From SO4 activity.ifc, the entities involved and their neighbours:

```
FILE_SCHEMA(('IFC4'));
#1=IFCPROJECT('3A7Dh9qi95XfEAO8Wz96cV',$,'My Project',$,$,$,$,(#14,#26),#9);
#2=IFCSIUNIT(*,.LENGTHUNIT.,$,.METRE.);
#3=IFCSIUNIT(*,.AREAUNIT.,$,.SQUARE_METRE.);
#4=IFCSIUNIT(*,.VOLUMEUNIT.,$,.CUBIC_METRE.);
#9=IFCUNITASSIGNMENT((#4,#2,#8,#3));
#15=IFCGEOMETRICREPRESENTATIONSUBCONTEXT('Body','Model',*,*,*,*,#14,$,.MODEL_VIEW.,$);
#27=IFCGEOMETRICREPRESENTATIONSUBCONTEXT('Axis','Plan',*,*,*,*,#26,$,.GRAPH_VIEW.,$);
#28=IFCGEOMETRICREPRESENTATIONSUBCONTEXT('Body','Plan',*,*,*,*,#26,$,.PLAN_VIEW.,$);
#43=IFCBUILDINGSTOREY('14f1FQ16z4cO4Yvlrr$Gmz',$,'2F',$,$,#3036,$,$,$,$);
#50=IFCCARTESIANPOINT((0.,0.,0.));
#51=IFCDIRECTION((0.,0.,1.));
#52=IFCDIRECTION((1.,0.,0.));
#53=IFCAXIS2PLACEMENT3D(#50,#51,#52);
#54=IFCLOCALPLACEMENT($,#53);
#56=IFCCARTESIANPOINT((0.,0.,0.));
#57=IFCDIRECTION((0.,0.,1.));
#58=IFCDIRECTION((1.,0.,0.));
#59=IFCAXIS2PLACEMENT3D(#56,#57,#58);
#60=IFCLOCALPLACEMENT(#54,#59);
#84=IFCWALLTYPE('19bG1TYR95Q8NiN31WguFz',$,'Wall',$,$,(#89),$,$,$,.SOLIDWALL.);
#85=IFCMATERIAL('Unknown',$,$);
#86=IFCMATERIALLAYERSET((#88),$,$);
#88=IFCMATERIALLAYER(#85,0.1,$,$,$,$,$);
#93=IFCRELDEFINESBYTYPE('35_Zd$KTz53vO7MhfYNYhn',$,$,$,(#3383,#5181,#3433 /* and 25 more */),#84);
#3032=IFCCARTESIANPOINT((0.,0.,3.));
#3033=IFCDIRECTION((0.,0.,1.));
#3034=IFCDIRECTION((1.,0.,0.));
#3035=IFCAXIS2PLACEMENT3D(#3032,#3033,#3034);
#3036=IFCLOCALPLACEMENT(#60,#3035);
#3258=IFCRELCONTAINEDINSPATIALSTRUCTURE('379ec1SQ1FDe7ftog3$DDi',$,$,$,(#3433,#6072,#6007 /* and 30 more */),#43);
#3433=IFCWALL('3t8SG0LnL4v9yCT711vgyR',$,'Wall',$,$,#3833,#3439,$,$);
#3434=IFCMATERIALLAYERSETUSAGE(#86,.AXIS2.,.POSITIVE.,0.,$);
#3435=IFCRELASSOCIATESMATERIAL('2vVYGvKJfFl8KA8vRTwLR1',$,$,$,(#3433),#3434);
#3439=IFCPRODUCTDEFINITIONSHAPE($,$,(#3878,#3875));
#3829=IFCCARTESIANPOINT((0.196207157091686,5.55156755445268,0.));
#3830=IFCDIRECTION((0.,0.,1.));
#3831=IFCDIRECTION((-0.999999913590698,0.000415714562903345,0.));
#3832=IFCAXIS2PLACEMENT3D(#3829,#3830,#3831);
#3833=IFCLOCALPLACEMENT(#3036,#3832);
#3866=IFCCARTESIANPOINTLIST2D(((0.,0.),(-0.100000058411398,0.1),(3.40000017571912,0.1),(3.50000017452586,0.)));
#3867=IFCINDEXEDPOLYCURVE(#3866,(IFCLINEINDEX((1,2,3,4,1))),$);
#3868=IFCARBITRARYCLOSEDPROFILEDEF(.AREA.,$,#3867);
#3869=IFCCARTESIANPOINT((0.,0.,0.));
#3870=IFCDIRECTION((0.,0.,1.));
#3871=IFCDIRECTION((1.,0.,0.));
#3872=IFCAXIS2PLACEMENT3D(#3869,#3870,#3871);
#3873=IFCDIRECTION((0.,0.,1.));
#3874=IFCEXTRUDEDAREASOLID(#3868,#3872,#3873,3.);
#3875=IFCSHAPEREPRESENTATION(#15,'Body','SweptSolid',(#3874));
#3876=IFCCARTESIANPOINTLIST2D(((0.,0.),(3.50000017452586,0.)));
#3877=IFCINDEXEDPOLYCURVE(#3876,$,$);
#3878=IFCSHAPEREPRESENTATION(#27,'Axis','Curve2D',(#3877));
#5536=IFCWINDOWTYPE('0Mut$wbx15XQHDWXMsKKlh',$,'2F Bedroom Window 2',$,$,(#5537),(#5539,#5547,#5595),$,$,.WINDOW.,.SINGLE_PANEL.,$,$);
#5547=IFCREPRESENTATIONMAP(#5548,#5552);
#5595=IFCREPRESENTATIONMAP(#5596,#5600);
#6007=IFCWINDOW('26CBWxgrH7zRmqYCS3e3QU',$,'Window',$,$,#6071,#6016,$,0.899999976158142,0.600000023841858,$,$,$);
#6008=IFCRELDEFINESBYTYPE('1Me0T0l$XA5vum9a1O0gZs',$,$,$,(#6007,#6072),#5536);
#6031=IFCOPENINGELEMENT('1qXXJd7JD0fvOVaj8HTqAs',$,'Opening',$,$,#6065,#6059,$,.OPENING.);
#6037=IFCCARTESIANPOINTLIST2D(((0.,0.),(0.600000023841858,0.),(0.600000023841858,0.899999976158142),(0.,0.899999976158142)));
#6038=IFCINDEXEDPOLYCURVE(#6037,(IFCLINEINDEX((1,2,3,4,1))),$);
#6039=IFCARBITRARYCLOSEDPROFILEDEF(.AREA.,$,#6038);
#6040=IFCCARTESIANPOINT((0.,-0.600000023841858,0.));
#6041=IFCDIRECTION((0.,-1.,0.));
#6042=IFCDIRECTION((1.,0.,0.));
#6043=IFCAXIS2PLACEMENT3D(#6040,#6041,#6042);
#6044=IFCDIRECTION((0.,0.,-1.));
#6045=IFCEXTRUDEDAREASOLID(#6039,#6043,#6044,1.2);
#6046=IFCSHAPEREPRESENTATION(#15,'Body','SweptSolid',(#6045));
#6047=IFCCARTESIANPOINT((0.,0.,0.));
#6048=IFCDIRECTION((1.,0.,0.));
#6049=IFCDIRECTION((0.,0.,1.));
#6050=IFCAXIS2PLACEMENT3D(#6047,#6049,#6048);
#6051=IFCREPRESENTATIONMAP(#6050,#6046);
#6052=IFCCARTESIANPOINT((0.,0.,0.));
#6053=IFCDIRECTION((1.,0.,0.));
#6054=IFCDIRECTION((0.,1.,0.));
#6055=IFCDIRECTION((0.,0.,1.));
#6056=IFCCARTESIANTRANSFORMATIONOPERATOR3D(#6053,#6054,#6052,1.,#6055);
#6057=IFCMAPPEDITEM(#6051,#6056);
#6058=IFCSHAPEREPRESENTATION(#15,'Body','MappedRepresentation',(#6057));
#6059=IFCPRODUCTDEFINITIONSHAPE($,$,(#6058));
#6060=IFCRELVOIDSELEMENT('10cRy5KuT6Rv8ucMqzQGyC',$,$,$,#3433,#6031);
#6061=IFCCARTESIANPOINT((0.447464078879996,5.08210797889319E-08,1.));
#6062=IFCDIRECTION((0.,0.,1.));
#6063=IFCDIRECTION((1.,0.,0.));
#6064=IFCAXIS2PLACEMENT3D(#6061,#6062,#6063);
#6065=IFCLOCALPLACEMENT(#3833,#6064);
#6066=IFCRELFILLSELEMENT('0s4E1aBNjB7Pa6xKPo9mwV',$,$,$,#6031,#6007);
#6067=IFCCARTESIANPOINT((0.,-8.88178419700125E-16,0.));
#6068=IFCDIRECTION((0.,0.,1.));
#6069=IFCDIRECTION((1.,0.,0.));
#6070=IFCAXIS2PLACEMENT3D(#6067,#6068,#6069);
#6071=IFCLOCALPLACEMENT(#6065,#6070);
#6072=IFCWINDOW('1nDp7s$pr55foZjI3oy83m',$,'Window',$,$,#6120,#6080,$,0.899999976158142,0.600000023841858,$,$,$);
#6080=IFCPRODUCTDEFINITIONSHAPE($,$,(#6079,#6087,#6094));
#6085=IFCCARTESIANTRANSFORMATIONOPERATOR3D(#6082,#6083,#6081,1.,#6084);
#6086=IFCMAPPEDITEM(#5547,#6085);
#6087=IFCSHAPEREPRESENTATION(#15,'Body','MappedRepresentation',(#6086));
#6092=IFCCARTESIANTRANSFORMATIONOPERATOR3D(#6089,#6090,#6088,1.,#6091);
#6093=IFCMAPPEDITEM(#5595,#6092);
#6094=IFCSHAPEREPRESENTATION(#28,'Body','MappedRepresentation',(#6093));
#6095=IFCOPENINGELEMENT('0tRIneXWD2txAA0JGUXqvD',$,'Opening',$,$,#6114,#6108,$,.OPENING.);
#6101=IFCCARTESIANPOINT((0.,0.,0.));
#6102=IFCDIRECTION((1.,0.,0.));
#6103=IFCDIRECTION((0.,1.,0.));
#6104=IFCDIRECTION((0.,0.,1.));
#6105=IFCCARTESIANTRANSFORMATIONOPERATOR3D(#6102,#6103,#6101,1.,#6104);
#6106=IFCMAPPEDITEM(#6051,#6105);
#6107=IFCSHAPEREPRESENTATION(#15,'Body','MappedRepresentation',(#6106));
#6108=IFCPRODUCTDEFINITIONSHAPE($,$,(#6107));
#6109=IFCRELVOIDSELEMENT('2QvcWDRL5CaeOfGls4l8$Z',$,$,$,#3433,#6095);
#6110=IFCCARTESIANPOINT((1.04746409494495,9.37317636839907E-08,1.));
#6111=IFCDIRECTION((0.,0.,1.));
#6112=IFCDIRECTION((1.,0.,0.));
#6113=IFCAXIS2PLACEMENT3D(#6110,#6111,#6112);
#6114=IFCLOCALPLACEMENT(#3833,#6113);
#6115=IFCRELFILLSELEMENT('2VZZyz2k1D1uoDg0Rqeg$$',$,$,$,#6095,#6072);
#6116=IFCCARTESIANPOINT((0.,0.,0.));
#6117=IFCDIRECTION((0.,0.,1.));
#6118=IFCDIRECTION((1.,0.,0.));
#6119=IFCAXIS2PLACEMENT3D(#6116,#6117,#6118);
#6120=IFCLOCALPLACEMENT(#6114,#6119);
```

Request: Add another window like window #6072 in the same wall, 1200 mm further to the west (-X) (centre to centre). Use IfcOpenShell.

```python
import ifcopenshell
import ifcopenshell.api.feature
import ifcopenshell.api.geometry
import ifcopenshell.api.root
import ifcopenshell.geom
import ifcopenshell.util.element
import ifcopenshell.util.placement
import ifcopenshell.util.shape
import ifcopenshell.util.unit

model = ifcopenshell.open("SO4 activity.ifc")
unit_scale = ifcopenshell.util.unit.calculate_unit_scale(model)
settings = ifcopenshell.geom.settings()


def volume(element):
    """Net volume in cubic metres, openings subtracted."""
    shape = ifcopenshell.geom.create_shape(settings, element)
    return ifcopenshell.util.shape.get_volume(shape.geometry)


window = model.by_id(6072)
opening = window.FillsVoids[0].RelatingOpeningElement
wall = opening.VoidsElements[0].RelatingBuildingElement
before = volume(wall)
shift = ifcopenshell.util.placement.get_local_placement(wall.ObjectPlacement)[:3, 0] * 1.2 / unit_scale

# copy_class copies the void relationship, type, container and properties, but no geometry.
new_opening = ifcopenshell.api.root.copy_class(model, product=opening)
new_opening.Representation = ifcopenshell.util.element.copy_deep(
    model, opening.Representation, exclude=["IfcGeometricRepresentationContext", "IfcRepresentationMap"]
)
new_window = ifcopenshell.api.root.copy_class(model, product=window)
new_window.Representation = ifcopenshell.util.element.copy_deep(
    model, window.Representation, exclude=["IfcGeometricRepresentationContext", "IfcRepresentationMap"]
)
ifcopenshell.api.feature.add_filling(model, opening=new_opening, element=new_window)

for old, new in ((opening, new_opening), (window, new_window)):
    matrix = ifcopenshell.util.placement.get_local_placement(old.ObjectPlacement)
    matrix[:3, 3] += shift
    ifcopenshell.api.geometry.edit_object_placement(model, product=new, matrix=matrix, is_si=False)

after = volume(wall)

print(f"wall volume {before:.3f} -> {after:.3f} m3")

model.write("SO4 activity_edited.ifc")
```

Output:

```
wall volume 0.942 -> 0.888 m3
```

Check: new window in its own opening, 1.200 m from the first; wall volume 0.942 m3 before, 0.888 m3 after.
